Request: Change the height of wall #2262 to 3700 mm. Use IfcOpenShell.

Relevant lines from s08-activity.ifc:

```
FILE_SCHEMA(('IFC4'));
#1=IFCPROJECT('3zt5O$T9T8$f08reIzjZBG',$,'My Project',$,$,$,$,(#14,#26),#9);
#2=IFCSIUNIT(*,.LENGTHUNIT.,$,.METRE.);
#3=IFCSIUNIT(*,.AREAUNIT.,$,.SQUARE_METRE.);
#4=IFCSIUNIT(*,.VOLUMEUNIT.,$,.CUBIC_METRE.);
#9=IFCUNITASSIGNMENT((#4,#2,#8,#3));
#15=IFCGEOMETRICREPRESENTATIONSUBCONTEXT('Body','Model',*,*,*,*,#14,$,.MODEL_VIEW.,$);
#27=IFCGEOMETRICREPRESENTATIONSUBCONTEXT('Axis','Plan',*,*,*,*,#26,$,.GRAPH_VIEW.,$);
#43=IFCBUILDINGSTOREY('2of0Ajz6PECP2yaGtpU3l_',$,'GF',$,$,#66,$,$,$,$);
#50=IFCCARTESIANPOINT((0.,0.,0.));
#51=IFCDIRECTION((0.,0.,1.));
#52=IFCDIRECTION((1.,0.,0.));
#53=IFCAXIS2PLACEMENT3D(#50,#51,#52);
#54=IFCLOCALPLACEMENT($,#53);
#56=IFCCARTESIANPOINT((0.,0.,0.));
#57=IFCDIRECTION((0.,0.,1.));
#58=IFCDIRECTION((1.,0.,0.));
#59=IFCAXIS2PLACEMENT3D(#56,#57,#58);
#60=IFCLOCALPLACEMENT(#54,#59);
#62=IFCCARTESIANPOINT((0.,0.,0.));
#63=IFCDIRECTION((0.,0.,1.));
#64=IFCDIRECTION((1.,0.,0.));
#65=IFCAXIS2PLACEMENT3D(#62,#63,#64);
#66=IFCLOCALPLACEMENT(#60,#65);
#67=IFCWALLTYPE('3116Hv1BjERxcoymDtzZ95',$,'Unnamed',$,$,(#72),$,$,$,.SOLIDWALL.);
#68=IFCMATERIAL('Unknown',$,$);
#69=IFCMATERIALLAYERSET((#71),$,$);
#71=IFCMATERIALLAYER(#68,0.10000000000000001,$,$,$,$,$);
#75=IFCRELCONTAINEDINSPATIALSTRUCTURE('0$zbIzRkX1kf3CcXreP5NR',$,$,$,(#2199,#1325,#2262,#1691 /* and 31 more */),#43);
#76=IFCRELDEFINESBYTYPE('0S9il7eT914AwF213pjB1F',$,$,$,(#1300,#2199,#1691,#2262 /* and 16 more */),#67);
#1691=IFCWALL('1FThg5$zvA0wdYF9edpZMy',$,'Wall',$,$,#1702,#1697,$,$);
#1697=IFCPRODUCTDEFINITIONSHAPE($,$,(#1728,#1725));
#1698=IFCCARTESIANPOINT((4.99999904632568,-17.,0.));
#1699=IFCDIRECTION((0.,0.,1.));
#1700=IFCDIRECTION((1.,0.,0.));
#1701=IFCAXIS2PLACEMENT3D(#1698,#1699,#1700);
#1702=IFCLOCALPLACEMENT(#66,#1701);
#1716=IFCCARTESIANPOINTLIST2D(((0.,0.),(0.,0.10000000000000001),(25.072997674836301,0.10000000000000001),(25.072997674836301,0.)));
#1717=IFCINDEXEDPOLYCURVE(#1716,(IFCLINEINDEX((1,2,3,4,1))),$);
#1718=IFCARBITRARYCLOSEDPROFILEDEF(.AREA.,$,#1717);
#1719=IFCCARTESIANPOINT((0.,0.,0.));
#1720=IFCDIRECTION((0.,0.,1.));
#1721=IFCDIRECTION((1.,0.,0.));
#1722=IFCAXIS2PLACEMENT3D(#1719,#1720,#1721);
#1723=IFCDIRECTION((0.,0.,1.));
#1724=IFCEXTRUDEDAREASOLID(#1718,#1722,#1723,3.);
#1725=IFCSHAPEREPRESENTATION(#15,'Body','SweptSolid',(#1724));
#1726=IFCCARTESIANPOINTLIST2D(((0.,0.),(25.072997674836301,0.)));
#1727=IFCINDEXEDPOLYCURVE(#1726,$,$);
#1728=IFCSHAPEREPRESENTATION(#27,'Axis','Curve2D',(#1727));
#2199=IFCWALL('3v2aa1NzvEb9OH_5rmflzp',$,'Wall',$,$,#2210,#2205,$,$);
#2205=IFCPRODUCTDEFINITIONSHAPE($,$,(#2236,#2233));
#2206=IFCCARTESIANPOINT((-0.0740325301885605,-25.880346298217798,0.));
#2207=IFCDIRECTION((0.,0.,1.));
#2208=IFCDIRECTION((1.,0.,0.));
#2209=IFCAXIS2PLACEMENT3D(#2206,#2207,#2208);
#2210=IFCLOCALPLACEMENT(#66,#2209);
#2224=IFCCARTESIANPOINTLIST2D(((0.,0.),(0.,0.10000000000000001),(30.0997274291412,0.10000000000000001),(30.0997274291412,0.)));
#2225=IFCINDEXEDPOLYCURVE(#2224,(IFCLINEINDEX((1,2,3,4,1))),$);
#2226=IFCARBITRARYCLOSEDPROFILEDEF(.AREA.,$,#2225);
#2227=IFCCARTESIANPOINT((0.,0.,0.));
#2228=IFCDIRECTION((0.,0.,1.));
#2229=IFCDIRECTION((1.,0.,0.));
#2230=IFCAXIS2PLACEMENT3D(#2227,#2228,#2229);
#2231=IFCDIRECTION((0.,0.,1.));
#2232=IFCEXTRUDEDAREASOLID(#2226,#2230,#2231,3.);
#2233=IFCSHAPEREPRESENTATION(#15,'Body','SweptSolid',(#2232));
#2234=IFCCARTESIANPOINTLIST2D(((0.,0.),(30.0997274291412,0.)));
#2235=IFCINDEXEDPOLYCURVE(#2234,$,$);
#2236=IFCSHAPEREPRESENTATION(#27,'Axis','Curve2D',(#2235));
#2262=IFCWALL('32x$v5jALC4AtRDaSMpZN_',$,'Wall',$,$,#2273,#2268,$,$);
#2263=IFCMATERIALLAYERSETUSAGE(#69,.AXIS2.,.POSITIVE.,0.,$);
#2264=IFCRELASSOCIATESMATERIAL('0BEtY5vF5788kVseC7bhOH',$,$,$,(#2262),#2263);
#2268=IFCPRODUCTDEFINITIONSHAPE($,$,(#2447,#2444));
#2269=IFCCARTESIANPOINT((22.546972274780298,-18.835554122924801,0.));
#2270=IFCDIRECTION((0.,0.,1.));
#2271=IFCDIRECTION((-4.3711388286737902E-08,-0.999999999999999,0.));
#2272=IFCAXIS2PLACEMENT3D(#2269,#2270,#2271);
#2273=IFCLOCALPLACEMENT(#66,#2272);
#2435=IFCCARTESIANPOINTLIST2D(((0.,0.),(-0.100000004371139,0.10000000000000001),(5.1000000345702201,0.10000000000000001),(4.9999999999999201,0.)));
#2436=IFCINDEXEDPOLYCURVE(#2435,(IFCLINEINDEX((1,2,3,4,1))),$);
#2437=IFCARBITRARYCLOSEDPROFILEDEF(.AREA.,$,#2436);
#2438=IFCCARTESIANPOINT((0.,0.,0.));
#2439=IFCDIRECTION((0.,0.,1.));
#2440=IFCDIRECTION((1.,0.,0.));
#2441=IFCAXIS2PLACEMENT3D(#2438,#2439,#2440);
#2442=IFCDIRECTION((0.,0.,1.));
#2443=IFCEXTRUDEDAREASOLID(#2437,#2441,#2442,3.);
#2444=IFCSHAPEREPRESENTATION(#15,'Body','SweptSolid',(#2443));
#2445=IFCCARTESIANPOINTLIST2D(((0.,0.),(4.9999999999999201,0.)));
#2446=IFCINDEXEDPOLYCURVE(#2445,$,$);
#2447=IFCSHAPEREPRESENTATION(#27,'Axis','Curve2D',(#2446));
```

```python
import ifcopenshell
import ifcopenshell.geom
import ifcopenshell.util.representation
import ifcopenshell.util.shape

model = ifcopenshell.open("s08-activity.ifc")
settings = ifcopenshell.geom.settings()


def volume(element):
    """Net volume in cubic metres, openings subtracted."""
    shape = ifcopenshell.geom.create_shape(settings, element)
    return ifcopenshell.util.shape.get_volume(shape.geometry)


wall = model.by_guid("32x$v5jALC4AtRDaSMpZN_")
before = volume(wall)

body = ifcopenshell.util.representation.get_representation(wall, "Model", "Body")
solid = body.Items[0]
old_height = solid.Depth
solid.Depth = 3.7
after = volume(wall)

print(f"height {old_height:g} -> {solid.Depth:g}, volume {before:.3f} -> {after:.3f} m3")

model.write("s08-activity_updated.ifc")
```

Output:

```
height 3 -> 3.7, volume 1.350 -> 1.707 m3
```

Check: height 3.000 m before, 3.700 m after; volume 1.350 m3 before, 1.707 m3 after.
